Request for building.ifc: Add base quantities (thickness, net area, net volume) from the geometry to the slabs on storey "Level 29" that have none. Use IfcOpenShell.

First a look at what the model holds.

```python
import ifcopenshell
import ifcopenshell.util.element
import ifcopenshell.util.unit

model = ifcopenshell.open("building.ifc")
print(model.schema)
for unit_type in ("LENGTHUNIT", "AREAUNIT", "VOLUMEUNIT"):
    print(unit_type, ifcopenshell.util.unit.calculate_unit_scale(model, unit_type))
storey = next(s for s in model.by_type("IfcBuildingStorey") if s.Name == "Level 29")
slabs = [e for e in ifcopenshell.util.element.get_decomposition(storey) if e.is_a("IfcSlab")]
for e in sorted(slabs, key=lambda e: e.id()):
    print(e.id(), e.is_a(), e.Name, list(ifcopenshell.util.element.get_psets(e, qtos_only=True)), sep=" | ")
```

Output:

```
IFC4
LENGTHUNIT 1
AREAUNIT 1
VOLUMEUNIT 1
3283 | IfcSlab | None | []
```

```python
import ifcopenshell
import ifcopenshell.api.pset
import ifcopenshell.geom
import ifcopenshell.util.element
import ifcopenshell.util.shape
import ifcopenshell.util.unit

model = ifcopenshell.open("building.ifc")
unit_scale = ifcopenshell.util.unit.calculate_unit_scale(model)
area_scale = ifcopenshell.util.unit.calculate_unit_scale(model, "AREAUNIT")
volume_scale = ifcopenshell.util.unit.calculate_unit_scale(model, "VOLUMEUNIT")
settings = ifcopenshell.geom.settings()

storey = next(s for s in model.by_type("IfcBuildingStorey") if s.Name == "Level 29")
slabs = [e for e in ifcopenshell.util.element.get_decomposition(storey) if e.is_a("IfcSlab")]

for e in sorted(slabs, key=lambda e: e.id()):
    if ifcopenshell.util.element.get_psets(e, qtos_only=True, should_inherit=False):
        continue
    # Geometry comes back in metres, in the element's own axes.
    shape = ifcopenshell.geom.create_shape(settings, e)
    values = {
        "Width": ifcopenshell.util.shape.get_z(shape.geometry) / unit_scale,
        "NetArea": ifcopenshell.util.shape.get_footprint_area(shape.geometry) / area_scale,
        "NetVolume": ifcopenshell.util.shape.get_volume(shape.geometry) / volume_scale,
    }
    qto = ifcopenshell.api.pset.add_qto(model, product=e, name="Qto_SlabBaseQuantities")
    ifcopenshell.api.pset.edit_qto(model, qto=qto, properties=values)
    print(e.id(), {k: round(v, 3) for k, v in values.items()})

model.write("building_rev.ifc")
```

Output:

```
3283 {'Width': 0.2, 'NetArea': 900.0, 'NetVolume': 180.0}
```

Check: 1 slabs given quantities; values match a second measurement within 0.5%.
